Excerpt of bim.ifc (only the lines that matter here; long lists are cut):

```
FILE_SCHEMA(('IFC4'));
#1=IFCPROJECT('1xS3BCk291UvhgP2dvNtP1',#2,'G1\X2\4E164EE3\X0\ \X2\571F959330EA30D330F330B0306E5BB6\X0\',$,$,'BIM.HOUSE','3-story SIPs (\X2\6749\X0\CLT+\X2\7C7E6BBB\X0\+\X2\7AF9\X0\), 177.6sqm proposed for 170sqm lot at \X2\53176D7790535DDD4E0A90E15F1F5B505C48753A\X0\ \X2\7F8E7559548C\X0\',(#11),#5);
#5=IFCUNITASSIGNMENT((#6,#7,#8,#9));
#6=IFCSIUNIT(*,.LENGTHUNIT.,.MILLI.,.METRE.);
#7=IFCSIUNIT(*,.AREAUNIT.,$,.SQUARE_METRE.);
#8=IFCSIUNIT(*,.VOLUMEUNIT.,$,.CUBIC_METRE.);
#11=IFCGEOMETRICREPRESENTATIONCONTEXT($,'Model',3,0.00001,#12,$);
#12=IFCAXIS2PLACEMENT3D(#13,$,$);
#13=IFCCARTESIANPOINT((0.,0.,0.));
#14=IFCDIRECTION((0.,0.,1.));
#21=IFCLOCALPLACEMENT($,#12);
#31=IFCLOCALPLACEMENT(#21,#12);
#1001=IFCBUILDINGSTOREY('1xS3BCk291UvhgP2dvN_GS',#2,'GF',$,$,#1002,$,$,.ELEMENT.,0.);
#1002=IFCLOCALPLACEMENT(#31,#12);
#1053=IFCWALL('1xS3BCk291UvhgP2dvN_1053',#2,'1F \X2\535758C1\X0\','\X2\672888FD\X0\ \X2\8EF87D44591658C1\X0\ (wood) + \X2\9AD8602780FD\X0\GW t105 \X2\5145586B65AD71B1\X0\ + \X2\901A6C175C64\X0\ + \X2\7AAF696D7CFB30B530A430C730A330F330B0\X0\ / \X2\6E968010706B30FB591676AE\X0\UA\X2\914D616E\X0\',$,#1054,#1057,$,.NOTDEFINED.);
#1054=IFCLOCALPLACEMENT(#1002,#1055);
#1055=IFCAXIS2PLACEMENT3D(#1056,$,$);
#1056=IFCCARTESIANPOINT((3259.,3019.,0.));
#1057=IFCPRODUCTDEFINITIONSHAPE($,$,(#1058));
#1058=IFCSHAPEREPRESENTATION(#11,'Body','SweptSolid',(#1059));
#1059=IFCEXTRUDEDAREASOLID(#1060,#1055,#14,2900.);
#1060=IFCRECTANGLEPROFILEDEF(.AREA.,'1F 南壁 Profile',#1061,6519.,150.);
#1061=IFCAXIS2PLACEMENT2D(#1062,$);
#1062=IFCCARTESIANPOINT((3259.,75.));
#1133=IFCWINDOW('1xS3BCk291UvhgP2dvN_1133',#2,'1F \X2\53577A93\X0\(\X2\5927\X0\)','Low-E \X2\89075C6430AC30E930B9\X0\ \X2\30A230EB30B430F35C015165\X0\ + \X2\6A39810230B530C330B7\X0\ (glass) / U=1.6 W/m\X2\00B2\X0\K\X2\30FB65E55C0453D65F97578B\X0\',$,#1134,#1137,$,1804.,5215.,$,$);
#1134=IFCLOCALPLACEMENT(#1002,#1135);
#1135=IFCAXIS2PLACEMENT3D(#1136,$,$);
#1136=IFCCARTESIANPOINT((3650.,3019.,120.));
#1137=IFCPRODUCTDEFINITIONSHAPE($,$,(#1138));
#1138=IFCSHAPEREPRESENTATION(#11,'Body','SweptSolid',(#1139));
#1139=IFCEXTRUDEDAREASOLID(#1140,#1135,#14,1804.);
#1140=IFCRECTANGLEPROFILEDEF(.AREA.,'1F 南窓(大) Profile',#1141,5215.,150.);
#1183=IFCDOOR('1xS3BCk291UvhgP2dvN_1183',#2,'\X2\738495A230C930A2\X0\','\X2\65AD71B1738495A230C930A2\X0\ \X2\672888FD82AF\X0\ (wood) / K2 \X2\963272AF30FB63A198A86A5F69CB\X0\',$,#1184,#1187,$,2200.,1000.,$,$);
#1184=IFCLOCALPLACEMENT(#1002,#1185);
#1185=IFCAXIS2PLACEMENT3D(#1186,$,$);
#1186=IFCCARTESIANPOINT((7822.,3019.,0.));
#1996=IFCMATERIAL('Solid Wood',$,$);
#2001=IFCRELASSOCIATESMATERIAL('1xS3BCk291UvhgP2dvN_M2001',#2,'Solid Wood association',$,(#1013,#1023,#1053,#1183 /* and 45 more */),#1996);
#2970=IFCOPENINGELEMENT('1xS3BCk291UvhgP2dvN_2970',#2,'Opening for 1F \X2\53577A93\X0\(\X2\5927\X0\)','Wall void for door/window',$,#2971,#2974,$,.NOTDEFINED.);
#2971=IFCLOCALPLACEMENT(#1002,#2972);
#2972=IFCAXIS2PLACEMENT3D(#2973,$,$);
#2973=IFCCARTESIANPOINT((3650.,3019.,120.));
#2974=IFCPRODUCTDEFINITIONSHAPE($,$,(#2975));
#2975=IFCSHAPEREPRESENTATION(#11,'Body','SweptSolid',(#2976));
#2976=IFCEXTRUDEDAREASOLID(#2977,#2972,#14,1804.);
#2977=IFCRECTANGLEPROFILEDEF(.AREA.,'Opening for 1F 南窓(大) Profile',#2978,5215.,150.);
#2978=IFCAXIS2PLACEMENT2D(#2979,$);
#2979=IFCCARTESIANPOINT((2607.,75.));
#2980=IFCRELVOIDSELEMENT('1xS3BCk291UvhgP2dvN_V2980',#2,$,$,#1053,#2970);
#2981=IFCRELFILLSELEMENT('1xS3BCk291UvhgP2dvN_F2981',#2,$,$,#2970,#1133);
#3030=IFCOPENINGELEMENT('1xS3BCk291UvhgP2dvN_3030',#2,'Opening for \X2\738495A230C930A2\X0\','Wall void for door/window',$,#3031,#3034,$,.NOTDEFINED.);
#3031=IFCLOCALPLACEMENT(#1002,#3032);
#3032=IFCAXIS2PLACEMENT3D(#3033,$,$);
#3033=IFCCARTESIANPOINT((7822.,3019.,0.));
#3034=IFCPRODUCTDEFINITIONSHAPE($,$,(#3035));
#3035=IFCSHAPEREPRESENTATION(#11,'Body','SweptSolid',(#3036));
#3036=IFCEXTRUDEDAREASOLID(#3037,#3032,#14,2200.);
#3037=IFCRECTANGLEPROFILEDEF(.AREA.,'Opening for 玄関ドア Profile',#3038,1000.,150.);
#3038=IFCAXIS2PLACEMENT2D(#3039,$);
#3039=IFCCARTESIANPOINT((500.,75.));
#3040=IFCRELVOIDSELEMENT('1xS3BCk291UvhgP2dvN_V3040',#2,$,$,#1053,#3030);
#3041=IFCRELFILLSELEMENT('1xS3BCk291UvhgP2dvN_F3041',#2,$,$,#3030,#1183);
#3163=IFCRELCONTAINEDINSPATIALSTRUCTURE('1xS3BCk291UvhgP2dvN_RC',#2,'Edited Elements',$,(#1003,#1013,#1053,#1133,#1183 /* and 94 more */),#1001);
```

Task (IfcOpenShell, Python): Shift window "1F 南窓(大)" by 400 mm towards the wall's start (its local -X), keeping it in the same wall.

```python
import ifcopenshell
import ifcopenshell.api.geometry
import ifcopenshell.util.placement
import ifcopenshell.util.unit

model = ifcopenshell.open("bim.ifc")
unit_scale = ifcopenshell.util.unit.calculate_unit_scale(model)

window = model.by_guid("1xS3BCk291UvhgP2dvN_1133")
opening = window.FillsVoids[0].RelatingOpeningElement
wall = opening.VoidsElements[0].RelatingBuildingElement

wall_matrix = ifcopenshell.util.placement.get_local_placement(wall.ObjectPlacement)
shift = wall_matrix[:3, 0] * -0.4 / unit_scale
before = ifcopenshell.util.placement.get_local_placement(window.ObjectPlacement)[:3, 3].copy()

# The window is not placed relative to its opening, so move both.
for product in (opening, window):
    matrix = ifcopenshell.util.placement.get_local_placement(product.ObjectPlacement)
    matrix[:3, 3] += shift
    ifcopenshell.api.geometry.edit_object_placement(model, product=product, matrix=matrix, is_si=False)

after = ifcopenshell.util.placement.get_local_placement(window.ObjectPlacement)[:3, 3]
print("window moved by", (after - before).round(3) + 0.0)

model.write("bim_updated.ifc")
```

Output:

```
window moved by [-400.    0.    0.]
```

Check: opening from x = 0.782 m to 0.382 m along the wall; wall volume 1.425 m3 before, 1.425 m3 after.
